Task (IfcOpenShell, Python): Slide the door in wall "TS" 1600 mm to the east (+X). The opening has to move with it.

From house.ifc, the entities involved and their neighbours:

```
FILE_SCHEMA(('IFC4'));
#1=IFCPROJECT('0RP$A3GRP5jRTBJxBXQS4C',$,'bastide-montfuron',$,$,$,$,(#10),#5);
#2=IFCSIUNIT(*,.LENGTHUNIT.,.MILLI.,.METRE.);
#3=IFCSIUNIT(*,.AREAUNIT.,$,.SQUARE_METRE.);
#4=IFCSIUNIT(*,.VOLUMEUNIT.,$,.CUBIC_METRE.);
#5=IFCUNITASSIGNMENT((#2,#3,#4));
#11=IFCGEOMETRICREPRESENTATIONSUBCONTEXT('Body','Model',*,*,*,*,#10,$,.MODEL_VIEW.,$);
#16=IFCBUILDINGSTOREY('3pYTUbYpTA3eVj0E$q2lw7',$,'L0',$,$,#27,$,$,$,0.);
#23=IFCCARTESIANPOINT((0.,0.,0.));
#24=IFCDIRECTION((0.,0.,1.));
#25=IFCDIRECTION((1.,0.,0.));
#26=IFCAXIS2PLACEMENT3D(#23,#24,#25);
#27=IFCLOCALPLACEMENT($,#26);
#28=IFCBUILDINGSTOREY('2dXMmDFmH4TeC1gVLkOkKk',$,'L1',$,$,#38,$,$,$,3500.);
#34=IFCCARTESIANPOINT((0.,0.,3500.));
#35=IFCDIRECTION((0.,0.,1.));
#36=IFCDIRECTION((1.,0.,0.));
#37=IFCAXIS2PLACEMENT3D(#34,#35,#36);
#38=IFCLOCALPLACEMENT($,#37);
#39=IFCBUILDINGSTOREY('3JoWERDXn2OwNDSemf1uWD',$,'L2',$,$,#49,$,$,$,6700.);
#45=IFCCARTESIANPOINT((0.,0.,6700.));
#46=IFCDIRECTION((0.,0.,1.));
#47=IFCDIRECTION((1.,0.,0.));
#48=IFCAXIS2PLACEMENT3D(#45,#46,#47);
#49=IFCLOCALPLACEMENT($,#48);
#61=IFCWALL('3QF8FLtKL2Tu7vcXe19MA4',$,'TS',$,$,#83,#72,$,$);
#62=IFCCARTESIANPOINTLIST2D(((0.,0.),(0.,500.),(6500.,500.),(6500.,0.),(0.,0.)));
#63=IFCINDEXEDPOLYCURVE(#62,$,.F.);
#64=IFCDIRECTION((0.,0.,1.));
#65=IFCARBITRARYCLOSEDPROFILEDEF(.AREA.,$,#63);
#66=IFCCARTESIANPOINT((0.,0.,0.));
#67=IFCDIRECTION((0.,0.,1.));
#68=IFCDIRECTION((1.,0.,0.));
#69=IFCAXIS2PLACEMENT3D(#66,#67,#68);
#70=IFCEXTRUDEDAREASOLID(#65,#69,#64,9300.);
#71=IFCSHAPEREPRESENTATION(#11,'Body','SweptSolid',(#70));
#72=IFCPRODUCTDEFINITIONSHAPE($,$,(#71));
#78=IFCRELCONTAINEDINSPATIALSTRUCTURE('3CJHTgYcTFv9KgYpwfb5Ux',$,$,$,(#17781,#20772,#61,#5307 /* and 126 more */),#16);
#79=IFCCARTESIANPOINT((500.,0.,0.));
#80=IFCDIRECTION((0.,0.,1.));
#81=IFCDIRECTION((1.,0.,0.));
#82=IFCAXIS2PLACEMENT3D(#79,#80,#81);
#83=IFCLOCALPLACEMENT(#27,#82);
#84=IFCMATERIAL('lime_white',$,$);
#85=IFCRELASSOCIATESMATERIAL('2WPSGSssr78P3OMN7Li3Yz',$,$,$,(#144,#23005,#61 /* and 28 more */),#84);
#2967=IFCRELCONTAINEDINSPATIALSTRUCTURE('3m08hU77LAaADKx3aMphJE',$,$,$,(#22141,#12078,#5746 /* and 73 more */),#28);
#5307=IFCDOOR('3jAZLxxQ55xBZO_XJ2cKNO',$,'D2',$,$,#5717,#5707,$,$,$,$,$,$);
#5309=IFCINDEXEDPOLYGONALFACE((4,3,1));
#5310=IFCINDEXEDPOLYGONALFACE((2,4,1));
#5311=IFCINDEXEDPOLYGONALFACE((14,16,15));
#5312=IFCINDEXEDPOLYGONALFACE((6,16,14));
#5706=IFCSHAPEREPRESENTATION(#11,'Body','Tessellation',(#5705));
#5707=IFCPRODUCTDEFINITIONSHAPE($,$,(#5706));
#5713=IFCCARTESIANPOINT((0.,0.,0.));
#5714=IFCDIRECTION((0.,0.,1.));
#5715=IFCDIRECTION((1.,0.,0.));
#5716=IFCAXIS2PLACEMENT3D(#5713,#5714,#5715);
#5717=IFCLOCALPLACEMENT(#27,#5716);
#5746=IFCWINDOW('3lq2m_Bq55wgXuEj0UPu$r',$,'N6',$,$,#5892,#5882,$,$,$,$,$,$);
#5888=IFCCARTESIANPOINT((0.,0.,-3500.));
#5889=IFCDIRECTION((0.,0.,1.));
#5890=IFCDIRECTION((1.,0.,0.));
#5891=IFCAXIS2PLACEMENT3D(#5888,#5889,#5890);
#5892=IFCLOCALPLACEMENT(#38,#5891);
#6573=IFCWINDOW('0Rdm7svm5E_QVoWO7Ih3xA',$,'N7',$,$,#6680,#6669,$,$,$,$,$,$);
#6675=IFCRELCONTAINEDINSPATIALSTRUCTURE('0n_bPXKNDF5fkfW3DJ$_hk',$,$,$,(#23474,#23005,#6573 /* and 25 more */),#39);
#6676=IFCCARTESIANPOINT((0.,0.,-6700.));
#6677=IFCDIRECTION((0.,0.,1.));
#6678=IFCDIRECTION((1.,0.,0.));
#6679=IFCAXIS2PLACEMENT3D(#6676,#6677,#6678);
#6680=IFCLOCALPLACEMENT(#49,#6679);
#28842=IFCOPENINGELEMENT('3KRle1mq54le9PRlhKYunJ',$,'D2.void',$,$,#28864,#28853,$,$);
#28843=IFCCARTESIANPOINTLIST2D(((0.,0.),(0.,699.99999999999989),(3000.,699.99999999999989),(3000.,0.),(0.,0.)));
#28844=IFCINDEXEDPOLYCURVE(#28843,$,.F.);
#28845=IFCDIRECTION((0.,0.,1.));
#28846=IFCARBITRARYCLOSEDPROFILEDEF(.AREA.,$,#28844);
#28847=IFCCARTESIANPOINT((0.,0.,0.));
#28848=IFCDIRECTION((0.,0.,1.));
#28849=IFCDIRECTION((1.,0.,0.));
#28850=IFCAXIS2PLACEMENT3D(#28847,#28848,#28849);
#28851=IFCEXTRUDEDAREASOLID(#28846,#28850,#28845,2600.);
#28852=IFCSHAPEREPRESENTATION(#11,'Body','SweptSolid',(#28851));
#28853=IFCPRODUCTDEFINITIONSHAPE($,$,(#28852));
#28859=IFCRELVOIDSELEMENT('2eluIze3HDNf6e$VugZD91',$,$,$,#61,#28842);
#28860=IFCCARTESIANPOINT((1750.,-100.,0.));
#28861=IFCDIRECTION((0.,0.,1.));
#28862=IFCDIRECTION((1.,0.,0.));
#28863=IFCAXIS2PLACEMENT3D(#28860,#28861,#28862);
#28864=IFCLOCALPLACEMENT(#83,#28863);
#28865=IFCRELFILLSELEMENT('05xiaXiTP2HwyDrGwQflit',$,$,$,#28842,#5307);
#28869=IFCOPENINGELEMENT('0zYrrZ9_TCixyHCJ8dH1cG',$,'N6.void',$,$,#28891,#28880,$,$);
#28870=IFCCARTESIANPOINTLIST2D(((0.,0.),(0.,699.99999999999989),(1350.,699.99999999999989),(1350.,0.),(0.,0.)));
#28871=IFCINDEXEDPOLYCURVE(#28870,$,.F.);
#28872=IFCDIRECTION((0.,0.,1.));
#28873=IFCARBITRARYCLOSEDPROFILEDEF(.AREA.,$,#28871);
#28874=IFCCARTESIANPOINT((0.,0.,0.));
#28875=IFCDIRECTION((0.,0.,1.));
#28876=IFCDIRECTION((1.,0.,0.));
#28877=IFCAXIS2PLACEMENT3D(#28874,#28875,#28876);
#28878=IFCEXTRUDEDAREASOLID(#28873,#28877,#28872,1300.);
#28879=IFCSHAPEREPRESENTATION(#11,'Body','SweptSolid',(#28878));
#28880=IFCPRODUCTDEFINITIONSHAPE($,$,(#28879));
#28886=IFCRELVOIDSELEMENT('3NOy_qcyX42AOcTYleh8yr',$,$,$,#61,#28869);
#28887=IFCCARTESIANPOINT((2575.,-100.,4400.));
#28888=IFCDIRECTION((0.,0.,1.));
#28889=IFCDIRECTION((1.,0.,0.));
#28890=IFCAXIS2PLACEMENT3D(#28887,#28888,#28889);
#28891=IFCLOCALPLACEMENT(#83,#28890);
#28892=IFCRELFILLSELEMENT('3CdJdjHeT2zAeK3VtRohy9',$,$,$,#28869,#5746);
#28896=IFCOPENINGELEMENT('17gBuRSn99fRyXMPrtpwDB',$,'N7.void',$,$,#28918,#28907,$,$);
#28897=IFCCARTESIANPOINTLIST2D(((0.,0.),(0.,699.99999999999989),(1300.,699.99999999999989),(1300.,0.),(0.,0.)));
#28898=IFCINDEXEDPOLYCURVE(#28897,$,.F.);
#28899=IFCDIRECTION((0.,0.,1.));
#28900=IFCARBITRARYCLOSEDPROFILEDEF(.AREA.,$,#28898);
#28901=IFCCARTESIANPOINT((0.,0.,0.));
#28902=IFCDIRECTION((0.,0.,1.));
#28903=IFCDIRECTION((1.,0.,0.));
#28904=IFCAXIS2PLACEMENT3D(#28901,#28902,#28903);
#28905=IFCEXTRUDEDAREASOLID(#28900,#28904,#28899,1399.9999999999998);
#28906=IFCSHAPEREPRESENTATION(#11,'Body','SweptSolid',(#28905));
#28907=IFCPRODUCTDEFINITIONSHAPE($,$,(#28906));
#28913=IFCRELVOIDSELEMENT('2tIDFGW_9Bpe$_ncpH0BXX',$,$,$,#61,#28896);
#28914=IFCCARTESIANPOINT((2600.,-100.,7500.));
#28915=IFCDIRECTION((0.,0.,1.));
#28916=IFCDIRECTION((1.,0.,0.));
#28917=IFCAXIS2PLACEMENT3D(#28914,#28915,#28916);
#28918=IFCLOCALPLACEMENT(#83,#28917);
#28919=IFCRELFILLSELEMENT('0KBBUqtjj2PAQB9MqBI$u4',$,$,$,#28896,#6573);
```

```python
import ifcopenshell
import ifcopenshell.api.geometry
import ifcopenshell.util.placement
import ifcopenshell.util.unit

model = ifcopenshell.open("house.ifc")
unit_scale = ifcopenshell.util.unit.calculate_unit_scale(model)

door = model.by_guid("3jAZLxxQ55xBZO_XJ2cKNO")
opening = door.FillsVoids[0].RelatingOpeningElement
wall = opening.VoidsElements[0].RelatingBuildingElement

wall_matrix = ifcopenshell.util.placement.get_local_placement(wall.ObjectPlacement)
shift = wall_matrix[:3, 0] * 1.6 / unit_scale
before = ifcopenshell.util.placement.get_local_placement(door.ObjectPlacement)[:3, 3].copy()

# The door is not placed relative to its opening, so move both.
for product in (opening, door):
    matrix = ifcopenshell.util.placement.get_local_placement(product.ObjectPlacement)
    matrix[:3, 3] += shift
    ifcopenshell.api.geometry.edit_object_placement(model, product=product, matrix=matrix, is_si=False)

after = ifcopenshell.util.placement.get_local_placement(door.ObjectPlacement)[:3, 3]
print("door moved by", (after - before).round(3) + 0.0)

model.write("house_rev.ifc")
```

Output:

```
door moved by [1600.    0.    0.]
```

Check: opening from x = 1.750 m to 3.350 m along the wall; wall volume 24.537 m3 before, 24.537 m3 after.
